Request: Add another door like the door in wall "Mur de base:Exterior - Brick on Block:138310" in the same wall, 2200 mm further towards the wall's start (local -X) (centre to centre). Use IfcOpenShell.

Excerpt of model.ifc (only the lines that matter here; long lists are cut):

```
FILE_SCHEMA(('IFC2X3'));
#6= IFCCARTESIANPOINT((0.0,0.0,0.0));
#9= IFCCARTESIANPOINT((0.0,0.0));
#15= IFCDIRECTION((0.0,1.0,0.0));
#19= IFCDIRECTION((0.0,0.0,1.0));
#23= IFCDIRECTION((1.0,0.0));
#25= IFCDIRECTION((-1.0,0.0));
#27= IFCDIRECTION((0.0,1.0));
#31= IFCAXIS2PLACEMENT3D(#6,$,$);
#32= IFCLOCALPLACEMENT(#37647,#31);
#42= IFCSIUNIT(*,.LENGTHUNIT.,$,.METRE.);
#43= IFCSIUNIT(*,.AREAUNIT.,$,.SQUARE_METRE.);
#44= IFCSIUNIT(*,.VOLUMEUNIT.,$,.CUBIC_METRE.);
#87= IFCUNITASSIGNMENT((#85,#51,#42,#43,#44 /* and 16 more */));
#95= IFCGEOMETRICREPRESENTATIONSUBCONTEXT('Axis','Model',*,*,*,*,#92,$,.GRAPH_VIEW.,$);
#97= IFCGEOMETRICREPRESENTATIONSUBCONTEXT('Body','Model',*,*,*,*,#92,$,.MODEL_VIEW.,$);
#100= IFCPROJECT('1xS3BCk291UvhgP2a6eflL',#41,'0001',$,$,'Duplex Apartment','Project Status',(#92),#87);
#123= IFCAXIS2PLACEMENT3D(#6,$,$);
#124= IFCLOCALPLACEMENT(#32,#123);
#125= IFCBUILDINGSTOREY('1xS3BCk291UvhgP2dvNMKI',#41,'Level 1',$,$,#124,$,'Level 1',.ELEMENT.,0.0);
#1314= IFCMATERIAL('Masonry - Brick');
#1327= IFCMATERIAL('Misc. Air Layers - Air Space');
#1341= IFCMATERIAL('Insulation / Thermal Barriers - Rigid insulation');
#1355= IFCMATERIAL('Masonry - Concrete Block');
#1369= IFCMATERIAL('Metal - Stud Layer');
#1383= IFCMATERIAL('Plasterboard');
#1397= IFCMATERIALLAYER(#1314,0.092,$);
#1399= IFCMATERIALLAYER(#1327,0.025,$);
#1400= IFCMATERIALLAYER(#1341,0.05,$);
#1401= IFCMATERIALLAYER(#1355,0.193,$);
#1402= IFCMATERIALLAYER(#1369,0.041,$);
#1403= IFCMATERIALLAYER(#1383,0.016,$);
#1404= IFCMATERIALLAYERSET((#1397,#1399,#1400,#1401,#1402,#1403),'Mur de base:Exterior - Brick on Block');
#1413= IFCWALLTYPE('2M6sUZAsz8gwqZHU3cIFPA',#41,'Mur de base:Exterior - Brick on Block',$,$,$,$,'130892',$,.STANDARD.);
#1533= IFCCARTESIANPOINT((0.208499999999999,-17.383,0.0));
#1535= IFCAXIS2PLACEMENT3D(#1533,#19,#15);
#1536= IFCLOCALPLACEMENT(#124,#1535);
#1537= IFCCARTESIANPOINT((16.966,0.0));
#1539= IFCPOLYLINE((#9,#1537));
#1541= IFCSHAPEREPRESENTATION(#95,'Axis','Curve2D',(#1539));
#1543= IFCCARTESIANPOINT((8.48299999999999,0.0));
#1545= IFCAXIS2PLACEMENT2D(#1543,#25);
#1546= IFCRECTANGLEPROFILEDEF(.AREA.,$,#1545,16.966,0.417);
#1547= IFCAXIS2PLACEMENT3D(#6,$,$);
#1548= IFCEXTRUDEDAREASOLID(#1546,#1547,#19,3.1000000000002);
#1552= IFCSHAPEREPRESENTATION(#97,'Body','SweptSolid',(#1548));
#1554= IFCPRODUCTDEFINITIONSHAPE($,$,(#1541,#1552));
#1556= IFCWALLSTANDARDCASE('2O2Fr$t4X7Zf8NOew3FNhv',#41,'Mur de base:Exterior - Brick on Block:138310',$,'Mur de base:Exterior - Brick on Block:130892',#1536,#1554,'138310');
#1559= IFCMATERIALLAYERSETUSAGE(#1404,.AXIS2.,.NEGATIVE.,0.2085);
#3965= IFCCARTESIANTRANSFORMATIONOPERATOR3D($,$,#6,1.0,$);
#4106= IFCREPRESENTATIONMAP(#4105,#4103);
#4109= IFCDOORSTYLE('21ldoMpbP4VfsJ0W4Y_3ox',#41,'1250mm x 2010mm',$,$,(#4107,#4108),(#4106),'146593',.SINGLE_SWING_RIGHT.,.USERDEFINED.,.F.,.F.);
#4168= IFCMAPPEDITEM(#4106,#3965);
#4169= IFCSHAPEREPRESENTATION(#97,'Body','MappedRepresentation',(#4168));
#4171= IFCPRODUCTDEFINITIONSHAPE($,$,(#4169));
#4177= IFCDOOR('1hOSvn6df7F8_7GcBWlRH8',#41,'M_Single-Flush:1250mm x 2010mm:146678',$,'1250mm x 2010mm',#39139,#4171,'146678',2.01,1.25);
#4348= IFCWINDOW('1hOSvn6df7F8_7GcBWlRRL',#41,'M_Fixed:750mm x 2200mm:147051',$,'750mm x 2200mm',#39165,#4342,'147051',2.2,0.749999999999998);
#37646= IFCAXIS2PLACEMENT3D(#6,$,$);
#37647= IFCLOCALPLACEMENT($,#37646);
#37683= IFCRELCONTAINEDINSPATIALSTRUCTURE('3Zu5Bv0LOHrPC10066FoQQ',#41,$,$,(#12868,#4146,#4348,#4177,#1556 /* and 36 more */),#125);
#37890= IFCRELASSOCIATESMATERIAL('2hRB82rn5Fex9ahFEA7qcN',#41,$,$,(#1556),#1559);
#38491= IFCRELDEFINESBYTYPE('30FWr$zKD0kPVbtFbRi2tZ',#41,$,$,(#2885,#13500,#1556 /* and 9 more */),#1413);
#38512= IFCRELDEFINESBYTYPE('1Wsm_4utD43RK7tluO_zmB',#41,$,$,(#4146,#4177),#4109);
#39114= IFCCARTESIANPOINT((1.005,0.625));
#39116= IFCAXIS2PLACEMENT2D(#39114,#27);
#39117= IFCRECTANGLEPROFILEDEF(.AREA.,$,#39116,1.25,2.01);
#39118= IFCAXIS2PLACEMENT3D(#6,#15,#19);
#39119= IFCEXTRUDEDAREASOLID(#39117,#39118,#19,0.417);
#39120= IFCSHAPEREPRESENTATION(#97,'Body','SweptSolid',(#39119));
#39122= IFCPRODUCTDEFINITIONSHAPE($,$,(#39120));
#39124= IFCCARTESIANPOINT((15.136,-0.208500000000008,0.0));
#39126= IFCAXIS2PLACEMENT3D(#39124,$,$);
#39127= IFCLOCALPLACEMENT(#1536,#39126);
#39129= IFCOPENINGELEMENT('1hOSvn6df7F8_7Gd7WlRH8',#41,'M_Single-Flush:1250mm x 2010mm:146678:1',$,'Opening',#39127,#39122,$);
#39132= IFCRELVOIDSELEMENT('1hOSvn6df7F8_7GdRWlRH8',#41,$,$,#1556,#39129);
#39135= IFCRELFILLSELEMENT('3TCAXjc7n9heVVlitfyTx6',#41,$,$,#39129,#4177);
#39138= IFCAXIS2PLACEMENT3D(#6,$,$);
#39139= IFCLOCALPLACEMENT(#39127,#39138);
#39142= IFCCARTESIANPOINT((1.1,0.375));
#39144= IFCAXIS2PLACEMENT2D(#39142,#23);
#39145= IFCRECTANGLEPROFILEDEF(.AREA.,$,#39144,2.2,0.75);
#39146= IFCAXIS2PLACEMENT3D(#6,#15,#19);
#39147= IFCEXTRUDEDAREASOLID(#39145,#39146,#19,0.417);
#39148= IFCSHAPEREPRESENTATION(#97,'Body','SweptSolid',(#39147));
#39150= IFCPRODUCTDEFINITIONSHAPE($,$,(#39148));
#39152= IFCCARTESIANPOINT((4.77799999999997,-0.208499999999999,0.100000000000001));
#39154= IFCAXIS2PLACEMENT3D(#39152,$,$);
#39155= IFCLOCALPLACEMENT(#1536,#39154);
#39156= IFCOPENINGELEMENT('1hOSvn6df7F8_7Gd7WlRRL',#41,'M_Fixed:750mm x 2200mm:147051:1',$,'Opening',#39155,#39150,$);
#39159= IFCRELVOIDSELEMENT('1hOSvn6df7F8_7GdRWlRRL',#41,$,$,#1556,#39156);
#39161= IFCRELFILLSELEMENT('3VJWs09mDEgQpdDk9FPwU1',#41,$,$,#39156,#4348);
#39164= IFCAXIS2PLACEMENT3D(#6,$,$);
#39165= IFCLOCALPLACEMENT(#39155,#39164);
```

```python
import ifcopenshell
import ifcopenshell.api.feature
import ifcopenshell.api.geometry
import ifcopenshell.api.root
import ifcopenshell.geom
import ifcopenshell.util.element
import ifcopenshell.util.placement
import ifcopenshell.util.shape
import ifcopenshell.util.unit

model = ifcopenshell.open("model.ifc")
unit_scale = ifcopenshell.util.unit.calculate_unit_scale(model)
settings = ifcopenshell.geom.settings()


def volume(element):
    """Net volume in cubic metres, openings subtracted."""
    shape = ifcopenshell.geom.create_shape(settings, element)
    return ifcopenshell.util.shape.get_volume(shape.geometry)


def reuse_history(source, copy):
    """copy_class also copies each property set's owner history, people and application; keep the originals."""
    for rel in copy.IsDefinedBy:
        if rel.is_a("IfcRelDefinesByProperties") and (history := rel.RelatingPropertyDefinition.OwnerHistory):
            rel.RelatingPropertyDefinition.OwnerHistory = source.OwnerHistory
            ifcopenshell.util.element.remove_deep2(model, history)


door = model.by_guid("1hOSvn6df7F8_7GcBWlRH8")
opening = door.FillsVoids[0].RelatingOpeningElement
wall = opening.VoidsElements[0].RelatingBuildingElement
before = volume(wall)
shift = ifcopenshell.util.placement.get_local_placement(wall.ObjectPlacement)[:3, 0] * -2.2 / unit_scale

# copy_class copies the void relationship, type, container and properties, but no geometry.
new_opening = ifcopenshell.api.root.copy_class(model, product=opening)
new_opening.Representation = ifcopenshell.util.element.copy_deep(
    model, opening.Representation, exclude=["IfcGeometricRepresentationContext", "IfcRepresentationMap"]
)
new_opening.Name = "M_Single-Flush:1250mm x 2010mm"
new_door = ifcopenshell.api.root.copy_class(model, product=door)
new_door.Representation = ifcopenshell.util.element.copy_deep(
    model, door.Representation, exclude=["IfcGeometricRepresentationContext", "IfcRepresentationMap"]
)
new_door.Name = "M_Single-Flush:1250mm x 2010mm"
new_door.Tag = None
reuse_history(door, new_door)
fills = ifcopenshell.api.feature.add_filling(model, opening=new_opening, element=new_door)
fills.OwnerHistory = new_door.OwnerHistory  # required in IFC2X3

for old, new in ((opening, new_opening), (door, new_door)):
    matrix = ifcopenshell.util.placement.get_local_placement(old.ObjectPlacement)
    matrix[:3, 3] += shift
    ifcopenshell.api.geometry.edit_object_placement(model, product=new, matrix=matrix, is_si=False)

after = volume(wall)

print(f"wall volume {before:.3f} -> {after:.3f} m3")

model.write("model_rev.ifc")
```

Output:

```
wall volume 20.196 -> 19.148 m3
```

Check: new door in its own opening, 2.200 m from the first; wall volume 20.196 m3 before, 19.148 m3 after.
